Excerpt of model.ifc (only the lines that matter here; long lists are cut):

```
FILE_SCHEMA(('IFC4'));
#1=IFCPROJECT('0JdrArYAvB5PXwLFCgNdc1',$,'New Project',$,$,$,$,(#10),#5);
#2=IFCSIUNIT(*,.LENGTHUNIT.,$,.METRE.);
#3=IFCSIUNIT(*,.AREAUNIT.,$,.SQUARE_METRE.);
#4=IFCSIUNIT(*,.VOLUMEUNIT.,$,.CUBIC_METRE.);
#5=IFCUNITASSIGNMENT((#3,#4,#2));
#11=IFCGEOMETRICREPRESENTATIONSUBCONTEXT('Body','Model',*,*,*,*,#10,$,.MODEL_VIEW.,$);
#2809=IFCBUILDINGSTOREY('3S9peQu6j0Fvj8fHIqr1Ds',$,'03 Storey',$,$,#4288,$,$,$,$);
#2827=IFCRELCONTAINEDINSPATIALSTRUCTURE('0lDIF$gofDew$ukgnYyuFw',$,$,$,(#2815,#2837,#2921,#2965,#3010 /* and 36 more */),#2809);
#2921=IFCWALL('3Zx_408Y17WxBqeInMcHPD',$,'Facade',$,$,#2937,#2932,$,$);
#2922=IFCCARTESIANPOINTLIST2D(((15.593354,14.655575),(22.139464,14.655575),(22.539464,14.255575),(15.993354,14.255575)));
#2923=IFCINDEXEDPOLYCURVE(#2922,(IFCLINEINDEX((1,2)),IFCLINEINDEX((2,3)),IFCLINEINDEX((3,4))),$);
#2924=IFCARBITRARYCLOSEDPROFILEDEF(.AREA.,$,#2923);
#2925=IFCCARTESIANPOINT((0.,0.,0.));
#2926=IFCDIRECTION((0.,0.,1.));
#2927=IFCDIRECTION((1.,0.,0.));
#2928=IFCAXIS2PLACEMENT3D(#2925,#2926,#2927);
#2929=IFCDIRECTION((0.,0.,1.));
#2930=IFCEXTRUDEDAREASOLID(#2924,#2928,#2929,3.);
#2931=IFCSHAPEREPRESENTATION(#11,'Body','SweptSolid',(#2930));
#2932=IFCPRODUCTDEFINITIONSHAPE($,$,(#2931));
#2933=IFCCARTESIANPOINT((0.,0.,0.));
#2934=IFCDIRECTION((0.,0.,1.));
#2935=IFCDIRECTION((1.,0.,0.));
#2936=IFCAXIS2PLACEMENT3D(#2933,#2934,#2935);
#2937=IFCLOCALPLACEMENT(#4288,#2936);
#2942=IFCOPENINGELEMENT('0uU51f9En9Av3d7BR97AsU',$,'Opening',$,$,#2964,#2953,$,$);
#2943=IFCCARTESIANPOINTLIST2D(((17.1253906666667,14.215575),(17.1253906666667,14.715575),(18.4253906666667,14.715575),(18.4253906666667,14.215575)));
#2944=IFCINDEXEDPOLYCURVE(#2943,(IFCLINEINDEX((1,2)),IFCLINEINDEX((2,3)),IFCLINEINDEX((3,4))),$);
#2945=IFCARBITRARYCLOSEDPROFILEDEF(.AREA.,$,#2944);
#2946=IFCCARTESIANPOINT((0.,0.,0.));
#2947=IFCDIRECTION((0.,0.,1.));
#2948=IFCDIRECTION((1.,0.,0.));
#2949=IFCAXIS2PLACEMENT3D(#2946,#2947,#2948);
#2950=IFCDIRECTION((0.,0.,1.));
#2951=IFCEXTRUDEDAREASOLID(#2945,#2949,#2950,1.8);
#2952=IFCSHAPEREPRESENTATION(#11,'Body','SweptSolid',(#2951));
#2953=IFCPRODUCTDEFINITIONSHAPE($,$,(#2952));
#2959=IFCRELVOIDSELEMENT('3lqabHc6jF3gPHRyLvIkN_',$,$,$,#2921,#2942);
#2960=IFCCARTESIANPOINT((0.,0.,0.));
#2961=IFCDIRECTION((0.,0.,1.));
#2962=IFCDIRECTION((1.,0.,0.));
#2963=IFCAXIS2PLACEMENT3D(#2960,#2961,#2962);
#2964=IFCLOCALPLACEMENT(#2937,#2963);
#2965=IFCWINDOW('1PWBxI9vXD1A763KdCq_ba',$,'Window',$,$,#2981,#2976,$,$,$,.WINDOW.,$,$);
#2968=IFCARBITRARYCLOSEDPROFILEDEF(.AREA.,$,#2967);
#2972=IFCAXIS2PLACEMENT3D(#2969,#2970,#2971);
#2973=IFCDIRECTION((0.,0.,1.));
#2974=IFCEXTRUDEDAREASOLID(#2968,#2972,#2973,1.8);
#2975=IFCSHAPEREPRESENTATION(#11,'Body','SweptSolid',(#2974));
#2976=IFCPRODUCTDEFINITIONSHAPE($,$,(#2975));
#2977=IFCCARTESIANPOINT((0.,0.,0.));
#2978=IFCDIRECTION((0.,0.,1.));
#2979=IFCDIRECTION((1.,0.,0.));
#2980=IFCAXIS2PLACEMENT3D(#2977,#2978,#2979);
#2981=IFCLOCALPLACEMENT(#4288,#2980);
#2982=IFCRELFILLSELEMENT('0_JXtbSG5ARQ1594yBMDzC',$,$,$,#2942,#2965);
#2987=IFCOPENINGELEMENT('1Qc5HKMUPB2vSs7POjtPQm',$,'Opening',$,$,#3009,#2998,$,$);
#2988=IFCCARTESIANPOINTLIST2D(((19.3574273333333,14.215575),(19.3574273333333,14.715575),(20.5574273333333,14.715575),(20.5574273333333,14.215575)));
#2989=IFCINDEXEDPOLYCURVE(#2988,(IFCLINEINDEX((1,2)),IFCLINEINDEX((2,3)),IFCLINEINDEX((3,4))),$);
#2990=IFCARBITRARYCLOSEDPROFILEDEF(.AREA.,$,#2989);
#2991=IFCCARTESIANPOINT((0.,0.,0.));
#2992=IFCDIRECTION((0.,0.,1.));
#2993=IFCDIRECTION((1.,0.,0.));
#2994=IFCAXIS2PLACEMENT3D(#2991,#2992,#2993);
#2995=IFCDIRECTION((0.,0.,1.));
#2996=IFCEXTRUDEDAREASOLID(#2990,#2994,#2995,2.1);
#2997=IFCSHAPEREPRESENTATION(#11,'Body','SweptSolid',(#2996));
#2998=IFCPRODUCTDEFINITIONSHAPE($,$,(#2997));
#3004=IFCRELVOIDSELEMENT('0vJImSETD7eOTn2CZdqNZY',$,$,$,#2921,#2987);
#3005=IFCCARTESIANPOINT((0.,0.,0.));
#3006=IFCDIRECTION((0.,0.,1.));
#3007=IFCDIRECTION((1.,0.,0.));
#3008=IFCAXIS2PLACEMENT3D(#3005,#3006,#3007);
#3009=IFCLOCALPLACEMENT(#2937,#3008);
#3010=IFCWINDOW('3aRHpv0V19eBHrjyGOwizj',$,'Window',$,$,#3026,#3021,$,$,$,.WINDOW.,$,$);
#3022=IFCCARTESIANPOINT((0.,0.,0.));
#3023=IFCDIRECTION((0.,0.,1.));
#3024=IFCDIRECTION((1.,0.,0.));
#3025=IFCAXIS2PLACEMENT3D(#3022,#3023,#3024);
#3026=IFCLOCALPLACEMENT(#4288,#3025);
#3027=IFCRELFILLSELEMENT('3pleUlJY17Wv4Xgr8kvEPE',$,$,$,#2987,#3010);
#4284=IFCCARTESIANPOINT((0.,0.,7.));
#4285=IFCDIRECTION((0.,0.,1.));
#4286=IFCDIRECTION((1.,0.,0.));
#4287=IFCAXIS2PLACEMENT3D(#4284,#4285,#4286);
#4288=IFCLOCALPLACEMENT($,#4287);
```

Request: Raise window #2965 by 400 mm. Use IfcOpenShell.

```python
import numpy as np
import ifcopenshell
import ifcopenshell.api.geometry
import ifcopenshell.util.placement
import ifcopenshell.util.unit

model = ifcopenshell.open("model.ifc")
unit_scale = ifcopenshell.util.unit.calculate_unit_scale(model)

window = model.by_id(2965)
opening = window.FillsVoids[0].RelatingOpeningElement
dz = 0.4 / unit_scale

shift = np.array([0.0, 0.0, dz])
# The window is not placed relative to its opening, so move both.
for product in (opening, window):
    matrix = ifcopenshell.util.placement.get_local_placement(product.ObjectPlacement)
    matrix[:3, 3] += shift
    ifcopenshell.api.geometry.edit_object_placement(model, product=product, matrix=matrix, is_si=False)

print(f"moved by {dz * unit_scale:+.3f} m")

model.write("model_v2.ifc")
```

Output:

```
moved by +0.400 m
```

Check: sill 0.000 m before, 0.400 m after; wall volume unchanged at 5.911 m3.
